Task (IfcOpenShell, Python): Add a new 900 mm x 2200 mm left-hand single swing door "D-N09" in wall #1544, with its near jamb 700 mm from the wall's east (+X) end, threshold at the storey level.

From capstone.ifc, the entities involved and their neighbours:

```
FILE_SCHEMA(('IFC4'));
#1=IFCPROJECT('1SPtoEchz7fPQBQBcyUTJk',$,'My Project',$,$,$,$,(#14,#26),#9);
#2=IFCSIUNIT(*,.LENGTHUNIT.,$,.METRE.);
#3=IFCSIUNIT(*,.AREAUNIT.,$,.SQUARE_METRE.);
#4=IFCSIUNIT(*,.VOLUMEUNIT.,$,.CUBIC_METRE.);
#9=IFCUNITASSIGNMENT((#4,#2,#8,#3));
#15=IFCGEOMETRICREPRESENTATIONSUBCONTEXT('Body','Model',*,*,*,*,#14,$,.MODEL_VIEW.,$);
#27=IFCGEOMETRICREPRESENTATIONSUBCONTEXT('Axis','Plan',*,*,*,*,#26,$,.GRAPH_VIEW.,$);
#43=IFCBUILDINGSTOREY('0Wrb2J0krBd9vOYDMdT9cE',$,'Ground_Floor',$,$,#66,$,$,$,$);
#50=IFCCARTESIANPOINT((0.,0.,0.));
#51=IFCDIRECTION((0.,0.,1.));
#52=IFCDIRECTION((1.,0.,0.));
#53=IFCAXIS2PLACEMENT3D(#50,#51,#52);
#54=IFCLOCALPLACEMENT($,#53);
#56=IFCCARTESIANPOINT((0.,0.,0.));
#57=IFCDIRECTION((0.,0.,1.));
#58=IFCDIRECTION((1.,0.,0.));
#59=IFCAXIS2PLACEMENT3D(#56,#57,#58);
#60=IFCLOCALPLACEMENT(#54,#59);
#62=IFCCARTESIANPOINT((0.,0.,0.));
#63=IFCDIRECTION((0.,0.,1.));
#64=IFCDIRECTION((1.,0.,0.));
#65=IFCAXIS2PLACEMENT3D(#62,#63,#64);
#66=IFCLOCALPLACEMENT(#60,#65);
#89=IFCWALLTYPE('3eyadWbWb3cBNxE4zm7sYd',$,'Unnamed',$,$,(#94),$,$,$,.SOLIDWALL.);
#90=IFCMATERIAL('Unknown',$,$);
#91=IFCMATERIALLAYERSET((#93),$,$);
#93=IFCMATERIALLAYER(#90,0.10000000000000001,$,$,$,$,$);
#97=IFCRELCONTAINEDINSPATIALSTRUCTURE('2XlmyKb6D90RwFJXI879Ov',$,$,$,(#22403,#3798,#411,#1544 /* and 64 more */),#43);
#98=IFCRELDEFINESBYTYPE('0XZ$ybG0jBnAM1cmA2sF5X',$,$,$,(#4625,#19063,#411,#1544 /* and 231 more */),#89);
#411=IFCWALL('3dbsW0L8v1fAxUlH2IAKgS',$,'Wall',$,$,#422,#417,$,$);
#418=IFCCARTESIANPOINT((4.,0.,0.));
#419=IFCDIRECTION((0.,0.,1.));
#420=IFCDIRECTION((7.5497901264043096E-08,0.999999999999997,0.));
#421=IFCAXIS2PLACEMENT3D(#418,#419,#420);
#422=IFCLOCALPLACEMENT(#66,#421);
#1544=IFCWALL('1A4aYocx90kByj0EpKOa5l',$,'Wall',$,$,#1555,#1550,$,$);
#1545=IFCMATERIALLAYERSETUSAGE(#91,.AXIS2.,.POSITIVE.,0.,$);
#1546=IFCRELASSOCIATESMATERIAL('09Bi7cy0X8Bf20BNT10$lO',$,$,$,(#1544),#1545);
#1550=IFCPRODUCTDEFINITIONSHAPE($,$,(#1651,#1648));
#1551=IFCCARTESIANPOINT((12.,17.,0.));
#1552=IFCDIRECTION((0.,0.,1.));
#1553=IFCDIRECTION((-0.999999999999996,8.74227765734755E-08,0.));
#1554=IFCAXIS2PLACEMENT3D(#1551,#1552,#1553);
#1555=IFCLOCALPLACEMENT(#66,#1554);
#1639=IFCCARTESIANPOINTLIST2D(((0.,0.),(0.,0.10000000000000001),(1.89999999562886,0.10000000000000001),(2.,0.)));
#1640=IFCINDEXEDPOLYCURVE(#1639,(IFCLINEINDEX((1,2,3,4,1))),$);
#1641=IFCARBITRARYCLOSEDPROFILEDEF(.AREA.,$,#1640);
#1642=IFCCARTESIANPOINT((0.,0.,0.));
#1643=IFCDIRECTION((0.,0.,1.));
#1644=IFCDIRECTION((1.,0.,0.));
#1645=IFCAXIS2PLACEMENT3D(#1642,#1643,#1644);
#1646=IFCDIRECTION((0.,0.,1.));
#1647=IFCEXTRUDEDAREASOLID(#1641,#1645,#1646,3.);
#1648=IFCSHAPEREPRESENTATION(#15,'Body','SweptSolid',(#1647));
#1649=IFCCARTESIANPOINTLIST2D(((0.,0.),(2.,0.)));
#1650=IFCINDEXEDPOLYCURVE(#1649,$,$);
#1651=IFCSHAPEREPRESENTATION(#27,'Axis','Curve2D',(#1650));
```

```python
import numpy as np
import ifcopenshell
import ifcopenshell.api.feature
import ifcopenshell.api.geometry
import ifcopenshell.api.root
import ifcopenshell.api.spatial
import ifcopenshell.geom
import ifcopenshell.util.element
import ifcopenshell.util.placement
import ifcopenshell.util.representation
import ifcopenshell.util.shape
import ifcopenshell.util.unit

model = ifcopenshell.open("capstone.ifc")
unit_scale = ifcopenshell.util.unit.calculate_unit_scale(model)
settings = ifcopenshell.geom.settings()


def volume(element):
    """Net volume in cubic metres, openings subtracted."""
    shape = ifcopenshell.geom.create_shape(settings, element)
    return ifcopenshell.util.shape.get_volume(shape.geometry)


wall = model.by_id(1544)
storey = ifcopenshell.util.element.get_container(wall, ifc_class="IfcBuildingStorey")
context = ifcopenshell.util.representation.get_context(model, "Model", "Body", "MODEL_VIEW")
before = volume(wall)

width, height, from_end, sill = 0.9, 2.2, 0.7, 0.0  # metres

# The wall runs along its own X axis, and the end named is its -X end.
wall_shape = ifcopenshell.geom.create_shape(settings, wall)
x, y, z = ifcopenshell.util.shape.get_vertices(wall_shape.geometry).T
start = x.min() + from_end
face, thickness = float(y.min()), float(y.max() - y.min())
wall_matrix = ifcopenshell.util.placement.get_local_placement(wall.ObjectPlacement)
level = ifcopenshell.util.placement.get_local_placement(storey.ObjectPlacement)[2, 3]


def in_wall(x, y):
    """Placement at x, y metres in the wall's axes, at sill height."""
    matrix = wall_matrix.copy()
    matrix[:, 3] = wall_matrix @ np.array([x / unit_scale, y / unit_scale, 0.0, 1.0])
    matrix[2, 3] = level + sill / unit_scale
    return matrix


# Opening: a box that overshoots both wall faces by 50 mm.
opening = ifcopenshell.api.root.create_entity(model, ifc_class="IfcOpeningElement", predefined_type="OPENING")
box = ifcopenshell.api.geometry.add_wall_representation(
    model, context=context, length=width, height=height, thickness=thickness + 0.1
)
ifcopenshell.api.geometry.assign_representation(model, product=opening, representation=box)
ifcopenshell.api.geometry.edit_object_placement(model, product=opening, matrix=in_wall(start, face - 0.05), is_si=False)
ifcopenshell.api.feature.add_feature(model, feature=opening, element=wall)

door = ifcopenshell.api.root.create_entity(model, ifc_class="IfcDoor", name="D-N09", predefined_type="DOOR")
door.OverallWidth, door.OverallHeight = width / unit_scale, height / unit_scale
door.OperationType = "SINGLE_SWING_LEFT"
body = ifcopenshell.api.geometry.add_door_representation(
    model,
    context=context,
    overall_width=door.OverallWidth,
    overall_height=door.OverallHeight,
    operation_type="SINGLE_SWING_LEFT",
    lining_properties={"LiningDepth": thickness / unit_scale, "ThresholdDepth": thickness / unit_scale},
)
ifcopenshell.api.geometry.assign_representation(model, product=door, representation=body)
ifcopenshell.api.spatial.assign_container(model, products=[door], relating_structure=storey)
ifcopenshell.api.feature.add_filling(model, opening=opening, element=door)

# The lining spans the wall, so the door starts at the wall face.
ifcopenshell.api.geometry.edit_object_placement(model, product=door, matrix=in_wall(start, face), is_si=False)

after = volume(wall)

print(f"wall volume {before:.3f} -> {after:.3f} m3")

model.write("capstone_updated.ifc")
```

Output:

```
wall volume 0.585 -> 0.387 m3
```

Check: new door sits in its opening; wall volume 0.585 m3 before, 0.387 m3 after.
